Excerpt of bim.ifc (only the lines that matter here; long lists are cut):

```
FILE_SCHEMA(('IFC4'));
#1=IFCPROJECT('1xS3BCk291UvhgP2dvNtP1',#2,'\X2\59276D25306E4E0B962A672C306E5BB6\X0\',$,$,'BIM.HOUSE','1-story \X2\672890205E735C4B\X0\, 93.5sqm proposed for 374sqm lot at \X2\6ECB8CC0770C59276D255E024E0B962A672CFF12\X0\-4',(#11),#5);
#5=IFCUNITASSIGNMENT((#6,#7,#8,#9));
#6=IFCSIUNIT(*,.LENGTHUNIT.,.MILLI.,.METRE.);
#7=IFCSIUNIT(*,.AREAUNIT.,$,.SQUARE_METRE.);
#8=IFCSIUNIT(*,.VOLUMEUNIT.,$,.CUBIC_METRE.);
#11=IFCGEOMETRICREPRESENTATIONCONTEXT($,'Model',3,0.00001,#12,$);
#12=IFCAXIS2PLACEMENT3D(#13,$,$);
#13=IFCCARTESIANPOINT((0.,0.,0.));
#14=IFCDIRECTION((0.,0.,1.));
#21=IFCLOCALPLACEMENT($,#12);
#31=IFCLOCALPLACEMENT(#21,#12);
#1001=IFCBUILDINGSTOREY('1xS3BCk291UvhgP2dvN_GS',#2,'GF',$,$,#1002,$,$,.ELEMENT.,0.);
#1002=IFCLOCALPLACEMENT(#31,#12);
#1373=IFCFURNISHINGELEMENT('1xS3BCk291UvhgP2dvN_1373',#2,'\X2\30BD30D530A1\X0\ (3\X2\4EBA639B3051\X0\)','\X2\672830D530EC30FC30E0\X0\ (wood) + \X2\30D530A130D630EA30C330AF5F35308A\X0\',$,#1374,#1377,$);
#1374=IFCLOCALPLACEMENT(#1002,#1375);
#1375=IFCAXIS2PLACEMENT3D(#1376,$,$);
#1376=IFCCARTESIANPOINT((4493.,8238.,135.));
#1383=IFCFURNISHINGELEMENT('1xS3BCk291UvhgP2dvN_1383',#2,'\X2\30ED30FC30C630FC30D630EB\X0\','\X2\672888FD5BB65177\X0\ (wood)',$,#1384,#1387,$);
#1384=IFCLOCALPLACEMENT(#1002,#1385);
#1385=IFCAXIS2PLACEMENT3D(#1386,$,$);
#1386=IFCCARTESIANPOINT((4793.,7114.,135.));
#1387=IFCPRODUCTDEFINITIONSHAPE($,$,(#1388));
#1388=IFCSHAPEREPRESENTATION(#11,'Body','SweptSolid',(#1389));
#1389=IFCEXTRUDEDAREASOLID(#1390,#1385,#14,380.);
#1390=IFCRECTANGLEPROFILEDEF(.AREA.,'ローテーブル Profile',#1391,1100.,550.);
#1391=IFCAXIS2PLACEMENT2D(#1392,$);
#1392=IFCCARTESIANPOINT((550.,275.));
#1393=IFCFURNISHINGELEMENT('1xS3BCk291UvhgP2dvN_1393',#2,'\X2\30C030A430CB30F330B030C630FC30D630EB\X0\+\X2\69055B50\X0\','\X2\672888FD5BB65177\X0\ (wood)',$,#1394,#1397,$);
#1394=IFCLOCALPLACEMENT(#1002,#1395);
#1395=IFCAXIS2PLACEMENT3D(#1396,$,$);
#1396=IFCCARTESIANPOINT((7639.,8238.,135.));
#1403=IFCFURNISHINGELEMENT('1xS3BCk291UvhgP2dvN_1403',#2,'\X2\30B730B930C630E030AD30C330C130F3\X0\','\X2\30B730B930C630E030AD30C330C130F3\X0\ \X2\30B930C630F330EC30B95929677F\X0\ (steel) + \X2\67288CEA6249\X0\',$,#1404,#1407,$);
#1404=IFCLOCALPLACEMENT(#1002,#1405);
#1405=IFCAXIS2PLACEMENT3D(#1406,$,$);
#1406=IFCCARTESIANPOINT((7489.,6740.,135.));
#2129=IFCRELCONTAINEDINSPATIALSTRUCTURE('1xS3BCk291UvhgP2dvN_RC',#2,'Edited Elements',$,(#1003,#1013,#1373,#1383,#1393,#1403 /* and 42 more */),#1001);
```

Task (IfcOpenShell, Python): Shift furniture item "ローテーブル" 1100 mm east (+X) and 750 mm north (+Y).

```python
import ifcopenshell
import ifcopenshell.api.geometry
import ifcopenshell.util.placement
import ifcopenshell.util.unit

model = ifcopenshell.open("bim.ifc")
unit_scale = ifcopenshell.util.unit.calculate_unit_scale(model)

item = model.by_guid("1xS3BCk291UvhgP2dvN_1383")
matrix = ifcopenshell.util.placement.get_local_placement(item.ObjectPlacement)
matrix[0, 3] += 1.1 / unit_scale
matrix[1, 3] += 0.75 / unit_scale
ifcopenshell.api.geometry.edit_object_placement(model, product=item, matrix=matrix, is_si=False)

print(ifcopenshell.util.placement.get_local_placement(item.ObjectPlacement).round(3) + 0.0)

model.write("bim_updated.ifc")
```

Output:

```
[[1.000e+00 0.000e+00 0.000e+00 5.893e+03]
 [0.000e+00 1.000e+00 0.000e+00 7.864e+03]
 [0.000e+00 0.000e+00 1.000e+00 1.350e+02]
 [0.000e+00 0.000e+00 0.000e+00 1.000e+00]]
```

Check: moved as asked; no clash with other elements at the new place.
